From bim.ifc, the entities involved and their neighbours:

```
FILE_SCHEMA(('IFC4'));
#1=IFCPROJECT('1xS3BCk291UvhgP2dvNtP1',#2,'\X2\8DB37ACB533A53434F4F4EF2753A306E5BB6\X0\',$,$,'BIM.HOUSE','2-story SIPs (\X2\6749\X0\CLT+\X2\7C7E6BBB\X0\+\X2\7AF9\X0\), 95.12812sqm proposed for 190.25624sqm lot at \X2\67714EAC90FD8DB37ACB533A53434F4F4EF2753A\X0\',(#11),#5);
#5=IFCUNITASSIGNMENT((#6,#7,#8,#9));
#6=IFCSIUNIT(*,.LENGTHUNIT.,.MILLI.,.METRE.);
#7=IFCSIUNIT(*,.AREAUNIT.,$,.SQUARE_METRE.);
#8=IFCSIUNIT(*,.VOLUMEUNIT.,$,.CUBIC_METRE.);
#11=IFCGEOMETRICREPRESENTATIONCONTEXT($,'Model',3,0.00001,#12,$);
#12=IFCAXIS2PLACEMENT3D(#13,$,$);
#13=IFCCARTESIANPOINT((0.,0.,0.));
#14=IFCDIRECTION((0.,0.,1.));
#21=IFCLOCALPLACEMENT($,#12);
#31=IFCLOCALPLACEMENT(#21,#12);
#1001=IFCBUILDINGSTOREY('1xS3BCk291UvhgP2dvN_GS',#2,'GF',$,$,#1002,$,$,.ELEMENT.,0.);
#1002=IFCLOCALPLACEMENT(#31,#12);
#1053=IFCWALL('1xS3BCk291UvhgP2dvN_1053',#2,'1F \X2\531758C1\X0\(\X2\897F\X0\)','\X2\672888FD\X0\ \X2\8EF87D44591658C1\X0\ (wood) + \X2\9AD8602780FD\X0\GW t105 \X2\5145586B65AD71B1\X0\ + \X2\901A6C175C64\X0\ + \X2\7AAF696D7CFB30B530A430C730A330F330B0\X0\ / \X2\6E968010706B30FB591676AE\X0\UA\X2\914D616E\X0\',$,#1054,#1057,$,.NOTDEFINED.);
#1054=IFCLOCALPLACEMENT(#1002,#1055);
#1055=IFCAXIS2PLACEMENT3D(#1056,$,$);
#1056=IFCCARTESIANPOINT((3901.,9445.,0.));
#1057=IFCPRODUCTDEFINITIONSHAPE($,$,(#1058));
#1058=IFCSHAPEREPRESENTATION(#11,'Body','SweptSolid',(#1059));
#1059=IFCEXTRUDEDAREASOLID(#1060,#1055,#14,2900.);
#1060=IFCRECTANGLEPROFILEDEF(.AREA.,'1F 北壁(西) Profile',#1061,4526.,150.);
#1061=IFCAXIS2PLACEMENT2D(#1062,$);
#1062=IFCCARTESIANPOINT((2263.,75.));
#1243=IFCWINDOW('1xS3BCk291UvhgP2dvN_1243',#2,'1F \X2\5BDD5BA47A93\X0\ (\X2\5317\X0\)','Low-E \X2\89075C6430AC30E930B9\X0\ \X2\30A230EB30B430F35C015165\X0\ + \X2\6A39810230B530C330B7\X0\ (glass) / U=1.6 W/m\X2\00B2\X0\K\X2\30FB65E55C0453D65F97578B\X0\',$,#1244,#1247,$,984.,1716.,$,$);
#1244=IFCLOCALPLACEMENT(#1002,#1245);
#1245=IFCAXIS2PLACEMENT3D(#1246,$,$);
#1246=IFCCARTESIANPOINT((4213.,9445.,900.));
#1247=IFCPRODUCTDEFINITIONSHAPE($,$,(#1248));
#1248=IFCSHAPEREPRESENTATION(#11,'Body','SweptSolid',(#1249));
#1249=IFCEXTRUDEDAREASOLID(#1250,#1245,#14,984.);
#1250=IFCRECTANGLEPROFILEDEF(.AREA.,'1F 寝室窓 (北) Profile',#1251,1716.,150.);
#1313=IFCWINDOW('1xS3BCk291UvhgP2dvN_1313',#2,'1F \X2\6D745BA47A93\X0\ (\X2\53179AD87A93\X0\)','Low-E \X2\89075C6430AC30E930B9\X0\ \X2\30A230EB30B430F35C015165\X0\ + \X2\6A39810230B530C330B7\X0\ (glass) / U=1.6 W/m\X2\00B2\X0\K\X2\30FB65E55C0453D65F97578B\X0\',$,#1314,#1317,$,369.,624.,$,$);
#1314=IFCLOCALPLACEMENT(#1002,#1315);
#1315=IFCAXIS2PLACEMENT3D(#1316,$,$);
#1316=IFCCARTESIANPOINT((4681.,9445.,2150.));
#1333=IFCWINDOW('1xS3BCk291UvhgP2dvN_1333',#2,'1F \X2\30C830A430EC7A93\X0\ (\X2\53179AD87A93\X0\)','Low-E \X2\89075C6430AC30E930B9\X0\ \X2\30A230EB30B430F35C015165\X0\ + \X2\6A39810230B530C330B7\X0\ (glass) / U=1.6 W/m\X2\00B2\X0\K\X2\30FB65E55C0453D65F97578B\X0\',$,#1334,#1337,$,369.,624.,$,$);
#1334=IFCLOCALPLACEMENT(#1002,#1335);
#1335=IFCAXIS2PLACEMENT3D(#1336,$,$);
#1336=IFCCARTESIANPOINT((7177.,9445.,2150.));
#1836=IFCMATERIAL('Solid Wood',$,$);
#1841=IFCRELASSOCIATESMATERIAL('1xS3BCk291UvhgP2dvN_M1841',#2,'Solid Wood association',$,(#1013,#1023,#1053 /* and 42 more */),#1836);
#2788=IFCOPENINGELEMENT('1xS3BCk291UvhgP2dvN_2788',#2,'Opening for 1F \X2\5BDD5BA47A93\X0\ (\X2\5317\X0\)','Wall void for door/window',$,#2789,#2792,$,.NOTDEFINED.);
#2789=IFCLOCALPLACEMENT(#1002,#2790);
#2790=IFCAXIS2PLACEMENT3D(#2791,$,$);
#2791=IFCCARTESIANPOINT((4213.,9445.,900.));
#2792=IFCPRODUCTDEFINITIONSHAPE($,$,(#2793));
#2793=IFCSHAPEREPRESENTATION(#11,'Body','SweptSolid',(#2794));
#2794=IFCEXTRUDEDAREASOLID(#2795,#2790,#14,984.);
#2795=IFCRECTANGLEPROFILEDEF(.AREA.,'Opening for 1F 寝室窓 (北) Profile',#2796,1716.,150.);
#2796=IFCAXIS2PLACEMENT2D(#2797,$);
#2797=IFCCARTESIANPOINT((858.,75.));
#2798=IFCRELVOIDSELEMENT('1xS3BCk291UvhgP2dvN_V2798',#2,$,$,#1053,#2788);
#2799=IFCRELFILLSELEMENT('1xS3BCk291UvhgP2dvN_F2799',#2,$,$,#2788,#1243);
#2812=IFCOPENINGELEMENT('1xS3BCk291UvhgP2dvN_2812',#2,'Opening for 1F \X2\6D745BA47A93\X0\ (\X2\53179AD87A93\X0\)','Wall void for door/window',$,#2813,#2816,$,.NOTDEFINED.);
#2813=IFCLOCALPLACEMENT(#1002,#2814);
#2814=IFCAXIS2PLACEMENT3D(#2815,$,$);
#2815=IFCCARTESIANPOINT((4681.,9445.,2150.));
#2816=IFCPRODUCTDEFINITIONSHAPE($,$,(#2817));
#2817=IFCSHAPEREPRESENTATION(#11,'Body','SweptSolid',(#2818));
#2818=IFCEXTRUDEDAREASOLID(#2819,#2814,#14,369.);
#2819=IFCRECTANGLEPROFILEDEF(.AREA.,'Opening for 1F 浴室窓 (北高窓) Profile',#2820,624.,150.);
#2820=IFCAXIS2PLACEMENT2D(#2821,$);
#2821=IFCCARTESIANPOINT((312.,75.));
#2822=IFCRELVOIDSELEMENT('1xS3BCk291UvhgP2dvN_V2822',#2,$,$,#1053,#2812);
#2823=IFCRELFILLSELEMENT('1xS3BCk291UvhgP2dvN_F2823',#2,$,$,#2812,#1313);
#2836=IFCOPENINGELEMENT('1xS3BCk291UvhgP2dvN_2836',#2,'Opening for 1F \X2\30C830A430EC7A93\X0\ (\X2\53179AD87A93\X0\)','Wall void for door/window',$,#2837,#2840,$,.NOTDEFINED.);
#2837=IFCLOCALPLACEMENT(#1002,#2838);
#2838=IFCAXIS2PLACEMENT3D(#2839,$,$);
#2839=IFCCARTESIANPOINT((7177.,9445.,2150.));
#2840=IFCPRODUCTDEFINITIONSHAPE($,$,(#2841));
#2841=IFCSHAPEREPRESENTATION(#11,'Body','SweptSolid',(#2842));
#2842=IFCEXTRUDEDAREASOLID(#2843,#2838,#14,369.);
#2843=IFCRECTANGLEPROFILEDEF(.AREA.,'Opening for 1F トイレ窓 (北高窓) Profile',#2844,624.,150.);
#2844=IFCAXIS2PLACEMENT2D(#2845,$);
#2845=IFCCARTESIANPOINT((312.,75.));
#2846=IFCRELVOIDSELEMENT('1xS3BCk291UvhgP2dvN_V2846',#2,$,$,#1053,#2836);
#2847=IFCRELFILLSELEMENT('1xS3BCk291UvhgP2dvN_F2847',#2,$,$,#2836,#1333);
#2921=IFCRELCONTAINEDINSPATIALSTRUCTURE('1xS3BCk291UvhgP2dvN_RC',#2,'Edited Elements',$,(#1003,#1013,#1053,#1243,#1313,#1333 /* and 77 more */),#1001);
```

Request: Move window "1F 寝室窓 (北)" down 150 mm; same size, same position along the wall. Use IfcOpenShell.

```python
import numpy as np
import ifcopenshell
import ifcopenshell.api.geometry
import ifcopenshell.util.placement
import ifcopenshell.util.unit

model = ifcopenshell.open("bim.ifc")
unit_scale = ifcopenshell.util.unit.calculate_unit_scale(model)

window = model.by_guid("1xS3BCk291UvhgP2dvN_1243")
opening = window.FillsVoids[0].RelatingOpeningElement
dz = -0.15 / unit_scale

shift = np.array([0.0, 0.0, dz])
# The window is not placed relative to its opening, so move both.
for product in (opening, window):
    matrix = ifcopenshell.util.placement.get_local_placement(product.ObjectPlacement)
    matrix[:3, 3] += shift
    ifcopenshell.api.geometry.edit_object_placement(model, product=product, matrix=matrix, is_si=False)

print(f"moved by {dz * unit_scale:+.3f} m")

model.write("bim_rev.ifc")
```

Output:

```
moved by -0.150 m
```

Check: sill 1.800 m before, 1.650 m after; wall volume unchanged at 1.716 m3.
